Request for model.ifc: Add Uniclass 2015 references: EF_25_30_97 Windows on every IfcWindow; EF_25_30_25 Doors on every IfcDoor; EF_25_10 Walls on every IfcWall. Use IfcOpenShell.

First a look at what the model holds.

```python
import ifcopenshell

model = ifcopenshell.open("model.ifc")
print(model.schema)
print("classifications:", [c.Name for c in model.by_type("IfcClassification")])
for ifc_class in ("IfcDoor", "IfcRoof", "IfcStair", "IfcWall", "IfcWindow"):
    print(ifc_class, len(model.by_type(ifc_class)))
```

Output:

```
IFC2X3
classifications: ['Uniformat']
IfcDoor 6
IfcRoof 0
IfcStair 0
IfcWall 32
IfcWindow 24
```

```python
import ifcopenshell
import ifcopenshell.api.classification

model = ifcopenshell.open("model.ifc")

# IFC2X3 requires Source and Edition and has no link from the project to the system.
system = model.create_entity("IfcClassification", Source="NBS", Edition="2015", Name="Uniclass 2015")

codes = {
    "IfcWindow": ("EF_25_30_97", "Windows"),
    "IfcDoor": ("EF_25_30_25", "Doors"),
    "IfcWall": ("EF_25_10", "Walls"),
}
for ifc_class, (code, name) in codes.items():
    products = model.by_type(ifc_class)
    ifcopenshell.api.classification.add_reference(
        model, products=products, classification=system, identification=code, name=name
    )
    print(code, len(products))

model.write("model_v2.ifc")
```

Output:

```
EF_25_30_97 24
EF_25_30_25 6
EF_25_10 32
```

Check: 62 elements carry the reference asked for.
